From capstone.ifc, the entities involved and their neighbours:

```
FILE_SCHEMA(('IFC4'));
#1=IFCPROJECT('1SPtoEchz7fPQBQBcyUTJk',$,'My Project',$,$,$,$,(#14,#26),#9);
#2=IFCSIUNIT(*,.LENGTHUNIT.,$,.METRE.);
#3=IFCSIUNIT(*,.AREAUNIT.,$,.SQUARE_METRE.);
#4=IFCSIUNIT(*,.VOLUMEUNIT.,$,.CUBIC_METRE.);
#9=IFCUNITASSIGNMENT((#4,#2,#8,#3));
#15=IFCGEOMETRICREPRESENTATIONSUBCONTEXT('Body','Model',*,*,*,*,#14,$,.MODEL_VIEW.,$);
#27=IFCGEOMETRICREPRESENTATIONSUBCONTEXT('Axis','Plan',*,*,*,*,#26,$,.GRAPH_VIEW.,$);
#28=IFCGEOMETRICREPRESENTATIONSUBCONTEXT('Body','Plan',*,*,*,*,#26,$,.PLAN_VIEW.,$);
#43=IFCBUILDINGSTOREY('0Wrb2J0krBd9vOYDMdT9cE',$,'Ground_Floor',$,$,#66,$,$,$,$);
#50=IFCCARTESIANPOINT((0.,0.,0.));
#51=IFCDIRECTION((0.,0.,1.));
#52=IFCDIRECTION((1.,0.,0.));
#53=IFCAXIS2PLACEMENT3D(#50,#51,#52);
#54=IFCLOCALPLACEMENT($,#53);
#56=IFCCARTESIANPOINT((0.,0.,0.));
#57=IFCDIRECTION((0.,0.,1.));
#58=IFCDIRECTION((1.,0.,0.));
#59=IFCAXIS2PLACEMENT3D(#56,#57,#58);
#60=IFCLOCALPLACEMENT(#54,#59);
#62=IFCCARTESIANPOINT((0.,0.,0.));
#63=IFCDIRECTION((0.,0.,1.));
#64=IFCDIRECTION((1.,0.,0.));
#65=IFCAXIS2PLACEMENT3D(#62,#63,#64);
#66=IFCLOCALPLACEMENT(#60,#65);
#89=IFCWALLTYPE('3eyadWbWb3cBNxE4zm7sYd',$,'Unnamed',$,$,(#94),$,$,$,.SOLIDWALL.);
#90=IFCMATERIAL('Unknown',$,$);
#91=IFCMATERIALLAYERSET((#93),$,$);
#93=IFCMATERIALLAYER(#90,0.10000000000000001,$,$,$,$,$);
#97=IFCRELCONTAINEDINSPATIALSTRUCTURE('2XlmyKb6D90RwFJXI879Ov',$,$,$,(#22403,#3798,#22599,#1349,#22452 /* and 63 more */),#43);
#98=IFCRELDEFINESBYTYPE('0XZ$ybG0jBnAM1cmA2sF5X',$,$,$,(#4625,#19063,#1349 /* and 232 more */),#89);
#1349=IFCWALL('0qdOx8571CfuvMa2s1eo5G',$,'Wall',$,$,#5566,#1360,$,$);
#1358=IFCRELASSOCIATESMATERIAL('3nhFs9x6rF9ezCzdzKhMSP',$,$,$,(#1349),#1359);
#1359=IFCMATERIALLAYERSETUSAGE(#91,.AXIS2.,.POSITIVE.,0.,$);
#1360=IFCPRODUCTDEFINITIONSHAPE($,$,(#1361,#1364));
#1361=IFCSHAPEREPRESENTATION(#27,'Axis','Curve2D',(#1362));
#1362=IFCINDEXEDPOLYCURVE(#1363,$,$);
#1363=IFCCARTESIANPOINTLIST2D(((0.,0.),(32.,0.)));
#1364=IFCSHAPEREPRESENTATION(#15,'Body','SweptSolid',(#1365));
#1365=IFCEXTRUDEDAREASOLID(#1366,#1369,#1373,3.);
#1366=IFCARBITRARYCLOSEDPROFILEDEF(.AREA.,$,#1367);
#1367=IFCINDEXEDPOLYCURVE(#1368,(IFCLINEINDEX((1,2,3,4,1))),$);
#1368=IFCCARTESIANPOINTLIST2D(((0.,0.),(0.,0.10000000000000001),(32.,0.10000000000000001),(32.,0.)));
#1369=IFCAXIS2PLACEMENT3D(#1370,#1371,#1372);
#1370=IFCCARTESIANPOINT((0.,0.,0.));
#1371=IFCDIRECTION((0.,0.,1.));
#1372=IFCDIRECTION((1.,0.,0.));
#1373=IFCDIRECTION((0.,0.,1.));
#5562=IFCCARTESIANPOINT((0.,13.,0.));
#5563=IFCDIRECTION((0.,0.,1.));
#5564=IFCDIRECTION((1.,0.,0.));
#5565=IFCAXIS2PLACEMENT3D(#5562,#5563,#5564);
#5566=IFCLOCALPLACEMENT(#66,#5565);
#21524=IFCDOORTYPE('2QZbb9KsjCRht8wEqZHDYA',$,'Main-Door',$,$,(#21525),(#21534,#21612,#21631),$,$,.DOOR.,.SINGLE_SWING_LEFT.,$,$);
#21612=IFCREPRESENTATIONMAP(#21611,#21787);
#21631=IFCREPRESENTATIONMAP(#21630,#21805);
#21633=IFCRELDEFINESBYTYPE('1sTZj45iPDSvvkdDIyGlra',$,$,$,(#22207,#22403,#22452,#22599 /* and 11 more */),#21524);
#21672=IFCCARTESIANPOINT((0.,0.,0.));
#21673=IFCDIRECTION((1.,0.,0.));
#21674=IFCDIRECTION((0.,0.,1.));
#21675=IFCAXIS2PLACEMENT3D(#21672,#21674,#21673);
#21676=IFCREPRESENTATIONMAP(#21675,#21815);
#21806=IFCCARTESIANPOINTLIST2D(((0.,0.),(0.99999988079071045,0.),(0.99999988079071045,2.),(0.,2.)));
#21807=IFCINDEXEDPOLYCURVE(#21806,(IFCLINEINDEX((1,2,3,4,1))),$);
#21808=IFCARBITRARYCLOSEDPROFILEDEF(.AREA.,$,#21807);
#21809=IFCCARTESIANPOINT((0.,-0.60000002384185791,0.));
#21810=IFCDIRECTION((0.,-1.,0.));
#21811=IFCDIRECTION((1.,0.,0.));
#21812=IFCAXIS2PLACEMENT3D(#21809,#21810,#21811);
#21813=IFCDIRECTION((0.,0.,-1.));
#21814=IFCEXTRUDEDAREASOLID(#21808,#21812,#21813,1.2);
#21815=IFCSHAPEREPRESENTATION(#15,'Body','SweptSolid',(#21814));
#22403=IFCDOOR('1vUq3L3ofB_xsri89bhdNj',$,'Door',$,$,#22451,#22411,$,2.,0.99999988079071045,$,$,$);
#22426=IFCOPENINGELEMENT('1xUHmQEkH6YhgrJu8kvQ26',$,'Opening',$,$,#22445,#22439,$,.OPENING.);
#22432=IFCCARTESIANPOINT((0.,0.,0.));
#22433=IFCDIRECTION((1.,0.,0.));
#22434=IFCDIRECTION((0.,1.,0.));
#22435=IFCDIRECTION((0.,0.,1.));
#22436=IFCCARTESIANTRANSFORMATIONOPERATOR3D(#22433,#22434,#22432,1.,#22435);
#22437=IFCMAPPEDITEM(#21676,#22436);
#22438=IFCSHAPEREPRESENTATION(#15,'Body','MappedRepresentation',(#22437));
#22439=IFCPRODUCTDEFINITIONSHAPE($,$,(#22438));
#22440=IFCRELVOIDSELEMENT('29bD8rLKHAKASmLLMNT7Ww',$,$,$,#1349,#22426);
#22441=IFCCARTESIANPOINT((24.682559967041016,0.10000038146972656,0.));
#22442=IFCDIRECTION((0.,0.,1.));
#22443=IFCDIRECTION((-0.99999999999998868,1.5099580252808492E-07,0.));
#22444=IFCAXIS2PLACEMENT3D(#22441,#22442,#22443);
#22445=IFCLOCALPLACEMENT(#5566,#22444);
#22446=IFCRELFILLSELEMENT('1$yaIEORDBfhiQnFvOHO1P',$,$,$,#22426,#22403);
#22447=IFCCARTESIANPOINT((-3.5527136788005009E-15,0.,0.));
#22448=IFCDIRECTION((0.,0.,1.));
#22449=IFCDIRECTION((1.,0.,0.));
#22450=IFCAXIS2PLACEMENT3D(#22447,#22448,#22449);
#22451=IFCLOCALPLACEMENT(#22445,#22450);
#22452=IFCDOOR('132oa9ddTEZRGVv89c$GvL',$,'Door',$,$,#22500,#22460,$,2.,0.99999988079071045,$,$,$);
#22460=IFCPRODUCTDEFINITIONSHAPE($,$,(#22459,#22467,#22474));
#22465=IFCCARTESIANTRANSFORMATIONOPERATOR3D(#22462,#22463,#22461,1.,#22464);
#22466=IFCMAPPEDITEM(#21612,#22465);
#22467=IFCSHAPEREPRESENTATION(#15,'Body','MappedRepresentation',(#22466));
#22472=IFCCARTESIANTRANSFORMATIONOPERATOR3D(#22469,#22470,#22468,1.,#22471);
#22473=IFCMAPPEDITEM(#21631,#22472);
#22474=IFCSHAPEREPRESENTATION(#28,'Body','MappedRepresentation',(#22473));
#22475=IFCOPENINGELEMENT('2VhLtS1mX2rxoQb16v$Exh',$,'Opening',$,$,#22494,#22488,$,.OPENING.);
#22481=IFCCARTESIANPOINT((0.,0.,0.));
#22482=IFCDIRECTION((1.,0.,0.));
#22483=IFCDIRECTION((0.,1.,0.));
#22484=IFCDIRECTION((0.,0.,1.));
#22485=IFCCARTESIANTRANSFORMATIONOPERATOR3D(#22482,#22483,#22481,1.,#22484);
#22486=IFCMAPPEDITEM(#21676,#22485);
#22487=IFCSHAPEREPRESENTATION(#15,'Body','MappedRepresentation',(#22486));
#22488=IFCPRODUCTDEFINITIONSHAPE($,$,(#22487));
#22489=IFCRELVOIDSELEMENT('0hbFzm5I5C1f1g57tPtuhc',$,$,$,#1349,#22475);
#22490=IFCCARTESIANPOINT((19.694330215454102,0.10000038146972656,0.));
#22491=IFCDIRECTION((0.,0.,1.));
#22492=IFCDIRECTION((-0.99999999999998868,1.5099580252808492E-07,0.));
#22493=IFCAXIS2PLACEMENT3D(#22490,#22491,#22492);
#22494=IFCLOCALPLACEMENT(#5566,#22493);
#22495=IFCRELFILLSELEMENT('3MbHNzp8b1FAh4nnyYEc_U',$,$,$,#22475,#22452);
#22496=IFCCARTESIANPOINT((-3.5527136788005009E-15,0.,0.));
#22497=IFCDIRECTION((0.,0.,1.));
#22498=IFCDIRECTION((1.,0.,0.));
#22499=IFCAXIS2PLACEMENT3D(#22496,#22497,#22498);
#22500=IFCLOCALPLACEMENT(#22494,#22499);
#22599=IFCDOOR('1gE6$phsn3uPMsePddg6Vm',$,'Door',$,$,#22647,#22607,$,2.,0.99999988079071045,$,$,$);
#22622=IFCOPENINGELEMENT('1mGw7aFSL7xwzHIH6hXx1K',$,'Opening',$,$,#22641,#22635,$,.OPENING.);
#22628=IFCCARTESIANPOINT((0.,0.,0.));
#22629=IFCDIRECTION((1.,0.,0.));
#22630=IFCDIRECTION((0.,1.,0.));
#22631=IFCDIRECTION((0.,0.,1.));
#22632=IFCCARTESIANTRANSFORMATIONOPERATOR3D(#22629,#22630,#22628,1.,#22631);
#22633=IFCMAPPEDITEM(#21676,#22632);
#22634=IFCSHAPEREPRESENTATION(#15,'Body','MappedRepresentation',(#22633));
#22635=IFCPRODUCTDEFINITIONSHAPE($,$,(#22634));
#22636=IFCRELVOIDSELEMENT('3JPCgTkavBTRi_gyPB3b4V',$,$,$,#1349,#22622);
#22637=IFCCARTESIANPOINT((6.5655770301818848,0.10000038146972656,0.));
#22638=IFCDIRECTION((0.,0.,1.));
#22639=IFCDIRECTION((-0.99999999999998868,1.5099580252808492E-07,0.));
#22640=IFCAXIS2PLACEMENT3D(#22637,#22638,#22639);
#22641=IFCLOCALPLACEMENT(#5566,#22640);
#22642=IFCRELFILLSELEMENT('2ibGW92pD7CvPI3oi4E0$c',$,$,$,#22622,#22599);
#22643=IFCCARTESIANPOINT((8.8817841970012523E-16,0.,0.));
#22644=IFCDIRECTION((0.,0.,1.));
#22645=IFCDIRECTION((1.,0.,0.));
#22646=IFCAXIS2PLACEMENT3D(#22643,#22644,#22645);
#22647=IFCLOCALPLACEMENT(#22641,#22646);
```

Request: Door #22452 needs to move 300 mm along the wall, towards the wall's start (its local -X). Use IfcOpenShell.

```python
import ifcopenshell
import ifcopenshell.api.geometry
import ifcopenshell.util.placement

model = ifcopenshell.open("capstone.ifc")

door = model.by_guid("132oa9ddTEZRGVv89c$GvL")
opening = door.FillsVoids[0].RelatingOpeningElement
wall = opening.VoidsElements[0].RelatingBuildingElement

wall_matrix = ifcopenshell.util.placement.get_local_placement(wall.ObjectPlacement)
shift = wall_matrix[:3, 0] * -0.3
before = ifcopenshell.util.placement.get_local_placement(door.ObjectPlacement)[:3, 3].copy()

# The door is placed relative to its opening, so it follows when the opening moves.
matrix = ifcopenshell.util.placement.get_local_placement(opening.ObjectPlacement)
matrix[:3, 3] += shift
ifcopenshell.api.geometry.edit_object_placement(
    model, product=opening, matrix=matrix, is_si=False, should_transform_children=True
)

after = ifcopenshell.util.placement.get_local_placement(door.ObjectPlacement)[:3, 3]
print("door moved by", (after - before).round(3) + 0.0)

model.write("capstone_edited.ifc")
```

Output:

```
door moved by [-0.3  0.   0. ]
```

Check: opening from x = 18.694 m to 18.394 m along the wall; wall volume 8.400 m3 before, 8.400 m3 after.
